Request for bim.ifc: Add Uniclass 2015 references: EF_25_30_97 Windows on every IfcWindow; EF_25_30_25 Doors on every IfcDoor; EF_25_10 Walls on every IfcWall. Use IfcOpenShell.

First a look at what the model holds.

```python
import ifcopenshell

model = ifcopenshell.open("bim.ifc")
print(model.schema)
print("classifications:", [c.Name for c in model.by_type("IfcClassification")])
for ifc_class in ("IfcDoor", "IfcRoof", "IfcStair", "IfcWall", "IfcWindow"):
    print(ifc_class, len(model.by_type(ifc_class)))
```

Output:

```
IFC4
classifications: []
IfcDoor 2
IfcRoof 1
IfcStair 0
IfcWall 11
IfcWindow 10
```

```python
import ifcopenshell
import ifcopenshell.api.classification

model = ifcopenshell.open("bim.ifc")

system = ifcopenshell.api.classification.add_classification(model, classification="Uniclass 2015")

codes = {
    "IfcWindow": ("EF_25_30_97", "Windows"),
    "IfcDoor": ("EF_25_30_25", "Doors"),
    "IfcWall": ("EF_25_10", "Walls"),
}
for ifc_class, (code, name) in codes.items():
    products = model.by_type(ifc_class)
    ifcopenshell.api.classification.add_reference(
        model, products=products, classification=system, identification=code, name=name
    )
    print(code, len(products))

model.write("bim_v2.ifc")
```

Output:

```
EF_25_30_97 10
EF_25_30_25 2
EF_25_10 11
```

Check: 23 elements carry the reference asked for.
